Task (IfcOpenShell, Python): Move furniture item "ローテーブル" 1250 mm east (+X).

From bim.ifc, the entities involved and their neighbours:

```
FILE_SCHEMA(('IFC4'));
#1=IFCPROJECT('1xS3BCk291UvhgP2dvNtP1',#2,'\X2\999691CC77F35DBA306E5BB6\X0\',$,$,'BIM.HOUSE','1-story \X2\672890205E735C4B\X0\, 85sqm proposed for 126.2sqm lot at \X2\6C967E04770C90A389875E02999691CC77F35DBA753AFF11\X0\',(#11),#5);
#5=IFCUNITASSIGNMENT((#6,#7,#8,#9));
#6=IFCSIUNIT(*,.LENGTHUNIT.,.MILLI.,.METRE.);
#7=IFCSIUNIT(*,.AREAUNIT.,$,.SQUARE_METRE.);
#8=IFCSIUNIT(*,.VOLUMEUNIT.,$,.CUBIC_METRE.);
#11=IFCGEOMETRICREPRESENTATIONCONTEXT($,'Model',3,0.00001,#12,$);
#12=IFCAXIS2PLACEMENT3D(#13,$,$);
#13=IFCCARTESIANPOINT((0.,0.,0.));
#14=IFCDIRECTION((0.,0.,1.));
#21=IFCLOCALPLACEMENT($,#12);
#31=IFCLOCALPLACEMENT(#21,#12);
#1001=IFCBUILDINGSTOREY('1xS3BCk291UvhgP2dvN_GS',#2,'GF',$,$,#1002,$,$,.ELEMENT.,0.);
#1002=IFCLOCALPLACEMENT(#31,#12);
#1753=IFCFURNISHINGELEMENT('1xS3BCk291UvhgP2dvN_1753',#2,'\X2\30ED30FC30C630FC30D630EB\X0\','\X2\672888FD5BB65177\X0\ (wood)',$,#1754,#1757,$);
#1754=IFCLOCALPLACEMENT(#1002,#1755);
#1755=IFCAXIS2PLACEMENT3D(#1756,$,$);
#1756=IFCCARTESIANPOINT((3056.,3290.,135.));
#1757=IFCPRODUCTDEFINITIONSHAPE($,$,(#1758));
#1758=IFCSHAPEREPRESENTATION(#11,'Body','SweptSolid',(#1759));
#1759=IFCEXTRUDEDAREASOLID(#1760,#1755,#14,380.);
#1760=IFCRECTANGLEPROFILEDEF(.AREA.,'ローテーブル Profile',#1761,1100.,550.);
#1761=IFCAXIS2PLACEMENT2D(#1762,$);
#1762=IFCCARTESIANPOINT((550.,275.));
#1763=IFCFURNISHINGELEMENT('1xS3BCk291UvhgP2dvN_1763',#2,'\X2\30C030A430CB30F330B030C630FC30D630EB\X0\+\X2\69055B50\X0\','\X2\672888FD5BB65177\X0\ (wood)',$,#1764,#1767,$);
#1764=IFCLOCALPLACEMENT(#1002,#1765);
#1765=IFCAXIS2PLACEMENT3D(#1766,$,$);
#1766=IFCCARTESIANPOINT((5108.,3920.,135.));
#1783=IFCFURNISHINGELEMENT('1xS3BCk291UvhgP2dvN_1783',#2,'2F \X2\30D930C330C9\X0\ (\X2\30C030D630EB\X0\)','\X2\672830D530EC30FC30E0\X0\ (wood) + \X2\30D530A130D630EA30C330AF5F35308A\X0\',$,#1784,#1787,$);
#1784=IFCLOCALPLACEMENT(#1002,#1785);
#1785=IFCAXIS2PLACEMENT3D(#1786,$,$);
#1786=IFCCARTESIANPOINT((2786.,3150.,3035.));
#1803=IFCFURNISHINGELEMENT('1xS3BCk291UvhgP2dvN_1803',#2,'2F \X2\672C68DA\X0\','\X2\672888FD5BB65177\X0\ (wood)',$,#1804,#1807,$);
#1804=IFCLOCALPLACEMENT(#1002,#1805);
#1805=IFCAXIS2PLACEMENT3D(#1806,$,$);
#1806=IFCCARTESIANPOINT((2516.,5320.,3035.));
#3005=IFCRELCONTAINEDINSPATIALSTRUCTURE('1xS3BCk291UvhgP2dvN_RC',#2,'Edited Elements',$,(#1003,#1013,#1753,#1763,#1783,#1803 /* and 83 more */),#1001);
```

```python
import ifcopenshell
import ifcopenshell.api.geometry
import ifcopenshell.util.placement

model = ifcopenshell.open("bim.ifc")

item = model.by_guid("1xS3BCk291UvhgP2dvN_1753")
matrix = ifcopenshell.util.placement.get_local_placement(item.ObjectPlacement)
matrix[0, 3] += 1250.0
ifcopenshell.api.geometry.edit_object_placement(model, product=item, matrix=matrix, is_si=False)

print(ifcopenshell.util.placement.get_local_placement(item.ObjectPlacement).round(3) + 0.0)

model.write("bim-out.ifc")
```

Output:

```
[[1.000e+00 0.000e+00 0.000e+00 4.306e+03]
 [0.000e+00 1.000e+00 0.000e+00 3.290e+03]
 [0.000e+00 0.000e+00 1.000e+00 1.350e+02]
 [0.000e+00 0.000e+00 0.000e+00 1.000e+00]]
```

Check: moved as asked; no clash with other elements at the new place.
